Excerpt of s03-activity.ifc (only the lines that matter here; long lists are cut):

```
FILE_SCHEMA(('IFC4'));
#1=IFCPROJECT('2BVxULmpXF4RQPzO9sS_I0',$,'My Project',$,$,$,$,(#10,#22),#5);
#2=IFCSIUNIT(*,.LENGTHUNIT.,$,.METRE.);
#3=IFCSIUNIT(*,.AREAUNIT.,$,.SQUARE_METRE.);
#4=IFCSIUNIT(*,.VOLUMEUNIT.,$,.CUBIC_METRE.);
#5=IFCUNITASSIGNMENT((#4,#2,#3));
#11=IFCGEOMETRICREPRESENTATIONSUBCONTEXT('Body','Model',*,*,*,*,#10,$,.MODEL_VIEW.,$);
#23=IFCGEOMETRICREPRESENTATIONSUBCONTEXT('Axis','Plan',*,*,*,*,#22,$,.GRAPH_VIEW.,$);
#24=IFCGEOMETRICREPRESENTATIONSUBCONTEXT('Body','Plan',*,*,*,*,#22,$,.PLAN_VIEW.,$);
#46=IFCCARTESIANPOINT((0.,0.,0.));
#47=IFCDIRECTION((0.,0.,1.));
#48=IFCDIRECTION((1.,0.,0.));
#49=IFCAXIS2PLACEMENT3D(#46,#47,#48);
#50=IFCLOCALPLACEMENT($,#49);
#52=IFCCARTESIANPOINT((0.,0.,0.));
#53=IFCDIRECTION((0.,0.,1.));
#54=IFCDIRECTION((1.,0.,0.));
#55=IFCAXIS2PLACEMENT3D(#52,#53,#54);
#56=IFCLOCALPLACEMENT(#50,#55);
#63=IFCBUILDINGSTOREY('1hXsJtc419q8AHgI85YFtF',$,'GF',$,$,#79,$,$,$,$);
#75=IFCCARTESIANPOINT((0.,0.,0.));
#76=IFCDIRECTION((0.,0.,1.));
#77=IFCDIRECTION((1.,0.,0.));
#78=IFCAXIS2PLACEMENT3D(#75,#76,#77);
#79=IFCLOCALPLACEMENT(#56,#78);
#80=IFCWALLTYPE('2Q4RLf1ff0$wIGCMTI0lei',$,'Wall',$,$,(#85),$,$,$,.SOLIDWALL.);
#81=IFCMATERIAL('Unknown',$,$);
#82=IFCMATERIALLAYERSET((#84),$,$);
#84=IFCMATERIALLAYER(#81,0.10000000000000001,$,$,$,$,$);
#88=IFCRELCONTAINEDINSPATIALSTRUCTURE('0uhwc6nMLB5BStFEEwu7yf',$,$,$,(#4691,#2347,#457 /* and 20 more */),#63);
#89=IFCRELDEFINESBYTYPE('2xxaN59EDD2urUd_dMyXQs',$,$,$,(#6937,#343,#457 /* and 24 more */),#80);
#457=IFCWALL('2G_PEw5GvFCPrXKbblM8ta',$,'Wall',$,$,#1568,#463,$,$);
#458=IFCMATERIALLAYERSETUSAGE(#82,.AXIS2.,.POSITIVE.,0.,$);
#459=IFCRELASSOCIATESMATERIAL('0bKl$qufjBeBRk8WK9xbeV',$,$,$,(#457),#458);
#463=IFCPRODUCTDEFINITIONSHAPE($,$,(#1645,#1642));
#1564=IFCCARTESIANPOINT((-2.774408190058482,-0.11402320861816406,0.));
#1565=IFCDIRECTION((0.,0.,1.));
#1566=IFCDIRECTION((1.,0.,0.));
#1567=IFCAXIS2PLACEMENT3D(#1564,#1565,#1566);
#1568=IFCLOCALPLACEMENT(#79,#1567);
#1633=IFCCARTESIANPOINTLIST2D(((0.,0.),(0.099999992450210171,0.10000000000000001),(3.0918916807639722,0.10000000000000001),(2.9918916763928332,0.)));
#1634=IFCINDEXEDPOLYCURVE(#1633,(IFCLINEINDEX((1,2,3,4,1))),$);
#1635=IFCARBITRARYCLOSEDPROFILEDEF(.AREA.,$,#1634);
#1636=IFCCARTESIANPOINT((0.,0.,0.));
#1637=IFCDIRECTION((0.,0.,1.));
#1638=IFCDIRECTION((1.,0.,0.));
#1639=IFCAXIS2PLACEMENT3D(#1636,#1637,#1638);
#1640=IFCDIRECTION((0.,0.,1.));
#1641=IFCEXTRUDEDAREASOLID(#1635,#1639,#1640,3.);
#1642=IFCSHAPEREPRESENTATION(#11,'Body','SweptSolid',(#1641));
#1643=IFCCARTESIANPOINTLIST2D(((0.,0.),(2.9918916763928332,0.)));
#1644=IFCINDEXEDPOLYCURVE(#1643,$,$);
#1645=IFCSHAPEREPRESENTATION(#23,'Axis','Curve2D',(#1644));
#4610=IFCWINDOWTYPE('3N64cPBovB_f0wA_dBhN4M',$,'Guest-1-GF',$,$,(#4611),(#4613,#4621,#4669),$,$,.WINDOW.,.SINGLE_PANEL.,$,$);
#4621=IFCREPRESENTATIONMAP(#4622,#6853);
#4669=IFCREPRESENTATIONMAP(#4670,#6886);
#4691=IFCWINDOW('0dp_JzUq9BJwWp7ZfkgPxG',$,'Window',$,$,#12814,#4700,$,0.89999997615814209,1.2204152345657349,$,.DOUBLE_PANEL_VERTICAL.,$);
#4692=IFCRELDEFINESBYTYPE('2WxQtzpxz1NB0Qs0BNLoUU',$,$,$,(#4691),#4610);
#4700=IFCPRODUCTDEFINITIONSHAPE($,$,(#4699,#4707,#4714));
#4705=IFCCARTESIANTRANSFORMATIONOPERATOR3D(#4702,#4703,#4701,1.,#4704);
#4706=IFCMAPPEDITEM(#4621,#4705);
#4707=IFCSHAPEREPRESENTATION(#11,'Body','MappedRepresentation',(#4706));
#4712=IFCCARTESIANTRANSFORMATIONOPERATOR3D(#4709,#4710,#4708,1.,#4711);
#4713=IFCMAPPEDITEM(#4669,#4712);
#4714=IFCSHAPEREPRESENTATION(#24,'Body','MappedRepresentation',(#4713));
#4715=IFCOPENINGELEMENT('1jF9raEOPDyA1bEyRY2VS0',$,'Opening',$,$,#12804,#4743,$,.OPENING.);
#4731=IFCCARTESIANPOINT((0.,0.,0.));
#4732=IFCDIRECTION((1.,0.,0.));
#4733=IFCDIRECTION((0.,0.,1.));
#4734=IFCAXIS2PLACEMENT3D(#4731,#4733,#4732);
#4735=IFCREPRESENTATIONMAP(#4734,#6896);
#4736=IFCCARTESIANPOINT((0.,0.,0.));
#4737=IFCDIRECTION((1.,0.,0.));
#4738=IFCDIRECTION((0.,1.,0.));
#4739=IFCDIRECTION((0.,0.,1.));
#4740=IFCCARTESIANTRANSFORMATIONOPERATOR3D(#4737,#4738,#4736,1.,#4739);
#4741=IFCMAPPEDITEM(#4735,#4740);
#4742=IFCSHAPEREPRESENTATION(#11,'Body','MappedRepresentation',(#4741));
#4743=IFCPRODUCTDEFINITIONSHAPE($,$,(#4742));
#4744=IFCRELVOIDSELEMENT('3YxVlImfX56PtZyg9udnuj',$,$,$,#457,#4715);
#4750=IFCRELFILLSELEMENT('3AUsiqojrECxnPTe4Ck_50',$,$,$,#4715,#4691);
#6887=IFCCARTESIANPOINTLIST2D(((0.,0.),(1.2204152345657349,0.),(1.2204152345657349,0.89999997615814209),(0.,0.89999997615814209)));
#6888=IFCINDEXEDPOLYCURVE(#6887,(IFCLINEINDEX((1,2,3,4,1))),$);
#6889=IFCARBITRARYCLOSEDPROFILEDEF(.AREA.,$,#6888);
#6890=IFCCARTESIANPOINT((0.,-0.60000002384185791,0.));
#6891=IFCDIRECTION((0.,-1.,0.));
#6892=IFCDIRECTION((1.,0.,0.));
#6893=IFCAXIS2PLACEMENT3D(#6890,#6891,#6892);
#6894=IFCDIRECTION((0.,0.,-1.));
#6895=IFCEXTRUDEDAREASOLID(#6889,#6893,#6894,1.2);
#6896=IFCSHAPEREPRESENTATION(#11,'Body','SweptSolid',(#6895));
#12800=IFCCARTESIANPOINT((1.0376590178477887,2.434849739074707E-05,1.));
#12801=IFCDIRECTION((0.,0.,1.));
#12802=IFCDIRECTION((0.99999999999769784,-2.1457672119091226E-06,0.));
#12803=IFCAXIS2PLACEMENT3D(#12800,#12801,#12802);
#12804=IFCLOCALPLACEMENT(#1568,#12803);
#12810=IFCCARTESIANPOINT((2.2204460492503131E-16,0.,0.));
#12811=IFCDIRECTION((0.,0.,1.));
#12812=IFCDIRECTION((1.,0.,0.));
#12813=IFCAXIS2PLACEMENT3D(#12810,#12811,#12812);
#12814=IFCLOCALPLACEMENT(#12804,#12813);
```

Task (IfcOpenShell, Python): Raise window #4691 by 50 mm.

```python
import numpy as np
import ifcopenshell
import ifcopenshell.api.geometry
import ifcopenshell.util.placement
import ifcopenshell.util.unit

model = ifcopenshell.open("s03-activity.ifc")
unit_scale = ifcopenshell.util.unit.calculate_unit_scale(model)

window = model.by_id(4691)
opening = window.FillsVoids[0].RelatingOpeningElement
dz = 0.05

shift = np.array([0.0, 0.0, dz])
# The window is placed relative to its opening, so it follows when the opening moves.
matrix = ifcopenshell.util.placement.get_local_placement(opening.ObjectPlacement)
matrix[:3, 3] += shift
ifcopenshell.api.geometry.edit_object_placement(
    model, product=opening, matrix=matrix, is_si=False, should_transform_children=True
)

print(f"moved by {dz * unit_scale:+.3f} m")

model.write("s03-activity-out.ifc")
```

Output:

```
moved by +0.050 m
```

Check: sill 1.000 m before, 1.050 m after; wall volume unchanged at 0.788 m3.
